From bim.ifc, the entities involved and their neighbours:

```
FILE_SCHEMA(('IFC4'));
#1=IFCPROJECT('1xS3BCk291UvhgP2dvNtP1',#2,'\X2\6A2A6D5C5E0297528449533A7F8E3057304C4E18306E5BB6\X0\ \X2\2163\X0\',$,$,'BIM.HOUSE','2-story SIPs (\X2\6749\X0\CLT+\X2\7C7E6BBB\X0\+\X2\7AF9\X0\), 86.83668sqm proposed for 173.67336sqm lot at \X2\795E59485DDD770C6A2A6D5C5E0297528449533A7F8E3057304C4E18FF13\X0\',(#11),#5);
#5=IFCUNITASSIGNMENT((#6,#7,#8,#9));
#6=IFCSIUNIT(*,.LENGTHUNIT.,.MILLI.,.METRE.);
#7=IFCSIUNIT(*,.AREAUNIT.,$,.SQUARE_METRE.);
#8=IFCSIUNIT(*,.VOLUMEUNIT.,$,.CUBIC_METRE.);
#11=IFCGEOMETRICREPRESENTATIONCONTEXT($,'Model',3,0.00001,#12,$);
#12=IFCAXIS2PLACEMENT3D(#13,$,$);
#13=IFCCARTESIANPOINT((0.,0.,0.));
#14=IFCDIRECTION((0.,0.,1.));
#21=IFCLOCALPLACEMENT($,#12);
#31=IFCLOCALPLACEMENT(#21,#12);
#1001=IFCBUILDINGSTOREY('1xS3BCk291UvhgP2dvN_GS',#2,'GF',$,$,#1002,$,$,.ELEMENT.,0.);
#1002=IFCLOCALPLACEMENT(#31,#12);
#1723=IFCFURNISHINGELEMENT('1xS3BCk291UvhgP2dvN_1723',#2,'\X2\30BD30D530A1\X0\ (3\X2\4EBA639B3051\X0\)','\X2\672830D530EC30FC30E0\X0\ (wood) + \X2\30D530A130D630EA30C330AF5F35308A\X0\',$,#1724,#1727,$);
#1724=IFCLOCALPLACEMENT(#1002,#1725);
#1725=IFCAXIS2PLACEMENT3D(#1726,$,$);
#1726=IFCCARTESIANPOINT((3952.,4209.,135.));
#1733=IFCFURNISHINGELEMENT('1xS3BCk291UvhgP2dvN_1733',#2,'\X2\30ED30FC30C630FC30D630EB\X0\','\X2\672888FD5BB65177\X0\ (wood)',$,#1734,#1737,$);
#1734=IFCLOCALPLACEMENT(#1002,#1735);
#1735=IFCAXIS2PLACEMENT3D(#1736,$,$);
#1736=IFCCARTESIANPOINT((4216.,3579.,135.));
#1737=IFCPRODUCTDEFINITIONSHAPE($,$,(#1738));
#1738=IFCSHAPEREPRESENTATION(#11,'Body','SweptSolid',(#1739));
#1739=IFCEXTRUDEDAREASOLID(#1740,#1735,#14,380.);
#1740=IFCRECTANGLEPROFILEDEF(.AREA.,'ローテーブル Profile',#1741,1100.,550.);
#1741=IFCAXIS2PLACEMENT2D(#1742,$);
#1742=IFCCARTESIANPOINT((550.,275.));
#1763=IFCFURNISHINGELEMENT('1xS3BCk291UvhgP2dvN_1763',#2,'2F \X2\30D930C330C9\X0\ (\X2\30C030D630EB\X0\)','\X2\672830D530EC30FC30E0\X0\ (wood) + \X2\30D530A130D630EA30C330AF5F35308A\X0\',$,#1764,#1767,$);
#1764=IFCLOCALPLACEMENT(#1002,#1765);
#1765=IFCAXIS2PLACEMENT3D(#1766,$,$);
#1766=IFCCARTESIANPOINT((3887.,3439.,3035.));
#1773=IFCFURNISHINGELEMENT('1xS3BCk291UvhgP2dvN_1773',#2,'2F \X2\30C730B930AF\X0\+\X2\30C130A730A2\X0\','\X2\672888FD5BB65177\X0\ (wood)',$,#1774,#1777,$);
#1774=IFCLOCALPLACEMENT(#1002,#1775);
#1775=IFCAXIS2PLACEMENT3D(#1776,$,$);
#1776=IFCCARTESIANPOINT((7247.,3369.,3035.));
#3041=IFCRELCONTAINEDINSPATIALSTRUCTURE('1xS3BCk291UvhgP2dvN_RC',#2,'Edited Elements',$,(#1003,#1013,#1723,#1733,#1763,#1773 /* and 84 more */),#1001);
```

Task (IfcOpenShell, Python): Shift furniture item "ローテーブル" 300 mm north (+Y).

```python
import ifcopenshell
import ifcopenshell.api.geometry
import ifcopenshell.util.placement
import ifcopenshell.util.unit

model = ifcopenshell.open("bim.ifc")
unit_scale = ifcopenshell.util.unit.calculate_unit_scale(model)

item = model.by_id(1733)
matrix = ifcopenshell.util.placement.get_local_placement(item.ObjectPlacement)
matrix[1, 3] += 0.3 / unit_scale
ifcopenshell.api.geometry.edit_object_placement(model, product=item, matrix=matrix, is_si=False)

print(ifcopenshell.util.placement.get_local_placement(item.ObjectPlacement).round(3) + 0.0)

model.write("bim-out.ifc")
```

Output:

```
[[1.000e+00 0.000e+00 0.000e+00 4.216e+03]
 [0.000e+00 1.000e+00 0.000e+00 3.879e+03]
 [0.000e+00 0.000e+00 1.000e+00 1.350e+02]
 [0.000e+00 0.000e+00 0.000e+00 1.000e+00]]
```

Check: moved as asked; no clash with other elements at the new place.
